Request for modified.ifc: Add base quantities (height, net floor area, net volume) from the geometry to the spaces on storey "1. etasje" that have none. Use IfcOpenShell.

First a look at what the model holds.

```python
import ifcopenshell
import ifcopenshell.util.element
import ifcopenshell.util.unit

model = ifcopenshell.open("modified.ifc")
print(model.schema)
for unit_type in ("LENGTHUNIT", "AREAUNIT", "VOLUMEUNIT"):
    print(unit_type, ifcopenshell.util.unit.calculate_unit_scale(model, unit_type))
storey = next(s for s in model.by_type("IfcBuildingStorey") if s.Name == "1. etasje")
spaces = [e for e in ifcopenshell.util.element.get_decomposition(storey) if e.is_a("IfcSpace")]
for e in sorted(spaces, key=lambda e: e.id()):
    print(e.id(), e.is_a(), e.Name, list(ifcopenshell.util.element.get_psets(e, qtos_only=True)), sep=" | ")
```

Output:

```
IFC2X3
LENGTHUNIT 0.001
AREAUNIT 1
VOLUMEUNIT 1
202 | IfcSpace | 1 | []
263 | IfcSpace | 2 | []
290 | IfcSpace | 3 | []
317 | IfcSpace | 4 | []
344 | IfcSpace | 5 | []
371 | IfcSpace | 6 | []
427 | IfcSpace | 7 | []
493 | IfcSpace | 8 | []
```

```python
import ifcopenshell
import ifcopenshell.api.pset
import ifcopenshell.geom
import ifcopenshell.util.element
import ifcopenshell.util.shape
import ifcopenshell.util.unit

model = ifcopenshell.open("modified.ifc")
unit_scale = ifcopenshell.util.unit.calculate_unit_scale(model)
area_scale = ifcopenshell.util.unit.calculate_unit_scale(model, "AREAUNIT")
volume_scale = ifcopenshell.util.unit.calculate_unit_scale(model, "VOLUMEUNIT")
settings = ifcopenshell.geom.settings()

storey = next(s for s in model.by_type("IfcBuildingStorey") if s.Name == "1. etasje")
spaces = [e for e in ifcopenshell.util.element.get_decomposition(storey) if e.is_a("IfcSpace")]

for e in sorted(spaces, key=lambda e: e.id()):
    if ifcopenshell.util.element.get_psets(e, qtos_only=True, should_inherit=False):
        continue
    # Geometry comes back in metres, in the element's own axes.
    shape = ifcopenshell.geom.create_shape(settings, e)
    values = {
        "Height": ifcopenshell.util.shape.get_z(shape.geometry) / unit_scale,
        "NetFloorArea": ifcopenshell.util.shape.get_footprint_area(shape.geometry) / area_scale,
        "NetVolume": ifcopenshell.util.shape.get_volume(shape.geometry) / volume_scale,
    }
    qto = ifcopenshell.api.pset.add_qto(model, product=e, name="BaseQuantities")
    ifcopenshell.api.pset.edit_qto(model, qto=qto, properties=values)
    print(e.id(), {k: round(v, 3) for k, v in values.items()})

model.write("modified_v2.ifc")
```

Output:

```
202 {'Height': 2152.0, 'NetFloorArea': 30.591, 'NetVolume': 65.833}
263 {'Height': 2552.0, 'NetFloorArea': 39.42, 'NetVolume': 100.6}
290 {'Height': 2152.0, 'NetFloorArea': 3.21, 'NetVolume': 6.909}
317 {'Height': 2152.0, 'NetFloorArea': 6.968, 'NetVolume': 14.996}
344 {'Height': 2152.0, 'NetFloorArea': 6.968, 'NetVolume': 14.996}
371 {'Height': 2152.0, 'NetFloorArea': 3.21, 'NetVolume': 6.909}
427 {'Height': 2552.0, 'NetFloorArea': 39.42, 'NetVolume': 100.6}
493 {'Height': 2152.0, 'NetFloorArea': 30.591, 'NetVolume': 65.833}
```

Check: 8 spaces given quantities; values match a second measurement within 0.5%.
